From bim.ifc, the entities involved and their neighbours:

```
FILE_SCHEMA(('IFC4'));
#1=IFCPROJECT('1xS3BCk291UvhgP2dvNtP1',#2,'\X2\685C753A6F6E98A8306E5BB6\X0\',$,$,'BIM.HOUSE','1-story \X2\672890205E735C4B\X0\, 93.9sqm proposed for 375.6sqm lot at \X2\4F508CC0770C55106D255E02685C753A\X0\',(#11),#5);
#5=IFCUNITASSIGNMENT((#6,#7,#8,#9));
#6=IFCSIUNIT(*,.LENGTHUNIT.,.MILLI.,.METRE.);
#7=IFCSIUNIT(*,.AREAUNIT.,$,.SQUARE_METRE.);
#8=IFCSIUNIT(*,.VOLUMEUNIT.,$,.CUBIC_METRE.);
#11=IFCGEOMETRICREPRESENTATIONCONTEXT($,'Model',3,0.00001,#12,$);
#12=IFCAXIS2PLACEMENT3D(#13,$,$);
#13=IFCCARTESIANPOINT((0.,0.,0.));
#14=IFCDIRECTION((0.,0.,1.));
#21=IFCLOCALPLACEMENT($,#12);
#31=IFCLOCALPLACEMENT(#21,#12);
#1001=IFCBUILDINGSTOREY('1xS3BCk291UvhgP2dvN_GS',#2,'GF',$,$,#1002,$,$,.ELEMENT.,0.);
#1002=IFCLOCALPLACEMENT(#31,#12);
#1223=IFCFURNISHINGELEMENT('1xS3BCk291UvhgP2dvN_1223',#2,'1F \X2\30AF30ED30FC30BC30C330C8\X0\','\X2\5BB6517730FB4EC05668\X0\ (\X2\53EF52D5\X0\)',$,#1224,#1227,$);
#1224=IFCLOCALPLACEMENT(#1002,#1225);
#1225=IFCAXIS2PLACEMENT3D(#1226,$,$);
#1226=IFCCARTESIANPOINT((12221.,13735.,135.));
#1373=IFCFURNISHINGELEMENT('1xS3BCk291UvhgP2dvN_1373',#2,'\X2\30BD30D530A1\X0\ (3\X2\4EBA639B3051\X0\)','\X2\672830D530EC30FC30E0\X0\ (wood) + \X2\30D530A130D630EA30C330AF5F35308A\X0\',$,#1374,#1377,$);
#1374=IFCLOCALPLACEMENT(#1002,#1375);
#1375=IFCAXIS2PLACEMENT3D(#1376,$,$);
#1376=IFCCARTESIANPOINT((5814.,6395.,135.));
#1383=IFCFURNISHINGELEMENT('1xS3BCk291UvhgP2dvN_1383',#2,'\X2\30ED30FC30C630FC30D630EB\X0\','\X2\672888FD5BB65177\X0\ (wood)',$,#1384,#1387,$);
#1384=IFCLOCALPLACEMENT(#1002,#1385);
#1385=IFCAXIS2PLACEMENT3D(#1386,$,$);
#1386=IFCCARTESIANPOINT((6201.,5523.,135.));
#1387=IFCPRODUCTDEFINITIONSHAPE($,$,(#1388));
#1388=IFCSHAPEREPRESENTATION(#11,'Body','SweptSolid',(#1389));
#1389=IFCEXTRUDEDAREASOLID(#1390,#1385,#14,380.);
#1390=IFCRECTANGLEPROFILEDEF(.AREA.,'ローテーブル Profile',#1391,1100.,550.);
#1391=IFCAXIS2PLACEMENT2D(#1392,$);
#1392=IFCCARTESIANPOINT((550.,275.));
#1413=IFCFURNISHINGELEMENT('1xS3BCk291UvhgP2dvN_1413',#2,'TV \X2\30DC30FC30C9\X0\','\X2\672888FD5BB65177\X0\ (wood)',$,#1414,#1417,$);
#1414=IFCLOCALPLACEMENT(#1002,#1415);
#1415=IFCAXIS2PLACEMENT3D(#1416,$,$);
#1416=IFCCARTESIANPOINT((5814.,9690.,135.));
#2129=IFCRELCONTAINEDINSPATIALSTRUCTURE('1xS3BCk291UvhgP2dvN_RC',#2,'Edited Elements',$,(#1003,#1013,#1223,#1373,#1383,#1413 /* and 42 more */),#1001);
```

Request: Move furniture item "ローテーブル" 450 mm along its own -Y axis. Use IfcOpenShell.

```python
import ifcopenshell
import ifcopenshell.api.geometry
import ifcopenshell.util.placement

model = ifcopenshell.open("bim.ifc")

item = model.by_guid("1xS3BCk291UvhgP2dvN_1383")
matrix = ifcopenshell.util.placement.get_local_placement(item.ObjectPlacement)
matrix[:3, 3] -= matrix[:3, 1] * 450.0
ifcopenshell.api.geometry.edit_object_placement(model, product=item, matrix=matrix, is_si=False)

print(ifcopenshell.util.placement.get_local_placement(item.ObjectPlacement).round(3) + 0.0)

model.write("bim_rev.ifc")
```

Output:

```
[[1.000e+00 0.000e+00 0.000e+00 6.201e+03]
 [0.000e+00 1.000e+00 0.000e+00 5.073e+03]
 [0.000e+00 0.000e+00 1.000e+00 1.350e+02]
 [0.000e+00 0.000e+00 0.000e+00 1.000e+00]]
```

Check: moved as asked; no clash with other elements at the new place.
